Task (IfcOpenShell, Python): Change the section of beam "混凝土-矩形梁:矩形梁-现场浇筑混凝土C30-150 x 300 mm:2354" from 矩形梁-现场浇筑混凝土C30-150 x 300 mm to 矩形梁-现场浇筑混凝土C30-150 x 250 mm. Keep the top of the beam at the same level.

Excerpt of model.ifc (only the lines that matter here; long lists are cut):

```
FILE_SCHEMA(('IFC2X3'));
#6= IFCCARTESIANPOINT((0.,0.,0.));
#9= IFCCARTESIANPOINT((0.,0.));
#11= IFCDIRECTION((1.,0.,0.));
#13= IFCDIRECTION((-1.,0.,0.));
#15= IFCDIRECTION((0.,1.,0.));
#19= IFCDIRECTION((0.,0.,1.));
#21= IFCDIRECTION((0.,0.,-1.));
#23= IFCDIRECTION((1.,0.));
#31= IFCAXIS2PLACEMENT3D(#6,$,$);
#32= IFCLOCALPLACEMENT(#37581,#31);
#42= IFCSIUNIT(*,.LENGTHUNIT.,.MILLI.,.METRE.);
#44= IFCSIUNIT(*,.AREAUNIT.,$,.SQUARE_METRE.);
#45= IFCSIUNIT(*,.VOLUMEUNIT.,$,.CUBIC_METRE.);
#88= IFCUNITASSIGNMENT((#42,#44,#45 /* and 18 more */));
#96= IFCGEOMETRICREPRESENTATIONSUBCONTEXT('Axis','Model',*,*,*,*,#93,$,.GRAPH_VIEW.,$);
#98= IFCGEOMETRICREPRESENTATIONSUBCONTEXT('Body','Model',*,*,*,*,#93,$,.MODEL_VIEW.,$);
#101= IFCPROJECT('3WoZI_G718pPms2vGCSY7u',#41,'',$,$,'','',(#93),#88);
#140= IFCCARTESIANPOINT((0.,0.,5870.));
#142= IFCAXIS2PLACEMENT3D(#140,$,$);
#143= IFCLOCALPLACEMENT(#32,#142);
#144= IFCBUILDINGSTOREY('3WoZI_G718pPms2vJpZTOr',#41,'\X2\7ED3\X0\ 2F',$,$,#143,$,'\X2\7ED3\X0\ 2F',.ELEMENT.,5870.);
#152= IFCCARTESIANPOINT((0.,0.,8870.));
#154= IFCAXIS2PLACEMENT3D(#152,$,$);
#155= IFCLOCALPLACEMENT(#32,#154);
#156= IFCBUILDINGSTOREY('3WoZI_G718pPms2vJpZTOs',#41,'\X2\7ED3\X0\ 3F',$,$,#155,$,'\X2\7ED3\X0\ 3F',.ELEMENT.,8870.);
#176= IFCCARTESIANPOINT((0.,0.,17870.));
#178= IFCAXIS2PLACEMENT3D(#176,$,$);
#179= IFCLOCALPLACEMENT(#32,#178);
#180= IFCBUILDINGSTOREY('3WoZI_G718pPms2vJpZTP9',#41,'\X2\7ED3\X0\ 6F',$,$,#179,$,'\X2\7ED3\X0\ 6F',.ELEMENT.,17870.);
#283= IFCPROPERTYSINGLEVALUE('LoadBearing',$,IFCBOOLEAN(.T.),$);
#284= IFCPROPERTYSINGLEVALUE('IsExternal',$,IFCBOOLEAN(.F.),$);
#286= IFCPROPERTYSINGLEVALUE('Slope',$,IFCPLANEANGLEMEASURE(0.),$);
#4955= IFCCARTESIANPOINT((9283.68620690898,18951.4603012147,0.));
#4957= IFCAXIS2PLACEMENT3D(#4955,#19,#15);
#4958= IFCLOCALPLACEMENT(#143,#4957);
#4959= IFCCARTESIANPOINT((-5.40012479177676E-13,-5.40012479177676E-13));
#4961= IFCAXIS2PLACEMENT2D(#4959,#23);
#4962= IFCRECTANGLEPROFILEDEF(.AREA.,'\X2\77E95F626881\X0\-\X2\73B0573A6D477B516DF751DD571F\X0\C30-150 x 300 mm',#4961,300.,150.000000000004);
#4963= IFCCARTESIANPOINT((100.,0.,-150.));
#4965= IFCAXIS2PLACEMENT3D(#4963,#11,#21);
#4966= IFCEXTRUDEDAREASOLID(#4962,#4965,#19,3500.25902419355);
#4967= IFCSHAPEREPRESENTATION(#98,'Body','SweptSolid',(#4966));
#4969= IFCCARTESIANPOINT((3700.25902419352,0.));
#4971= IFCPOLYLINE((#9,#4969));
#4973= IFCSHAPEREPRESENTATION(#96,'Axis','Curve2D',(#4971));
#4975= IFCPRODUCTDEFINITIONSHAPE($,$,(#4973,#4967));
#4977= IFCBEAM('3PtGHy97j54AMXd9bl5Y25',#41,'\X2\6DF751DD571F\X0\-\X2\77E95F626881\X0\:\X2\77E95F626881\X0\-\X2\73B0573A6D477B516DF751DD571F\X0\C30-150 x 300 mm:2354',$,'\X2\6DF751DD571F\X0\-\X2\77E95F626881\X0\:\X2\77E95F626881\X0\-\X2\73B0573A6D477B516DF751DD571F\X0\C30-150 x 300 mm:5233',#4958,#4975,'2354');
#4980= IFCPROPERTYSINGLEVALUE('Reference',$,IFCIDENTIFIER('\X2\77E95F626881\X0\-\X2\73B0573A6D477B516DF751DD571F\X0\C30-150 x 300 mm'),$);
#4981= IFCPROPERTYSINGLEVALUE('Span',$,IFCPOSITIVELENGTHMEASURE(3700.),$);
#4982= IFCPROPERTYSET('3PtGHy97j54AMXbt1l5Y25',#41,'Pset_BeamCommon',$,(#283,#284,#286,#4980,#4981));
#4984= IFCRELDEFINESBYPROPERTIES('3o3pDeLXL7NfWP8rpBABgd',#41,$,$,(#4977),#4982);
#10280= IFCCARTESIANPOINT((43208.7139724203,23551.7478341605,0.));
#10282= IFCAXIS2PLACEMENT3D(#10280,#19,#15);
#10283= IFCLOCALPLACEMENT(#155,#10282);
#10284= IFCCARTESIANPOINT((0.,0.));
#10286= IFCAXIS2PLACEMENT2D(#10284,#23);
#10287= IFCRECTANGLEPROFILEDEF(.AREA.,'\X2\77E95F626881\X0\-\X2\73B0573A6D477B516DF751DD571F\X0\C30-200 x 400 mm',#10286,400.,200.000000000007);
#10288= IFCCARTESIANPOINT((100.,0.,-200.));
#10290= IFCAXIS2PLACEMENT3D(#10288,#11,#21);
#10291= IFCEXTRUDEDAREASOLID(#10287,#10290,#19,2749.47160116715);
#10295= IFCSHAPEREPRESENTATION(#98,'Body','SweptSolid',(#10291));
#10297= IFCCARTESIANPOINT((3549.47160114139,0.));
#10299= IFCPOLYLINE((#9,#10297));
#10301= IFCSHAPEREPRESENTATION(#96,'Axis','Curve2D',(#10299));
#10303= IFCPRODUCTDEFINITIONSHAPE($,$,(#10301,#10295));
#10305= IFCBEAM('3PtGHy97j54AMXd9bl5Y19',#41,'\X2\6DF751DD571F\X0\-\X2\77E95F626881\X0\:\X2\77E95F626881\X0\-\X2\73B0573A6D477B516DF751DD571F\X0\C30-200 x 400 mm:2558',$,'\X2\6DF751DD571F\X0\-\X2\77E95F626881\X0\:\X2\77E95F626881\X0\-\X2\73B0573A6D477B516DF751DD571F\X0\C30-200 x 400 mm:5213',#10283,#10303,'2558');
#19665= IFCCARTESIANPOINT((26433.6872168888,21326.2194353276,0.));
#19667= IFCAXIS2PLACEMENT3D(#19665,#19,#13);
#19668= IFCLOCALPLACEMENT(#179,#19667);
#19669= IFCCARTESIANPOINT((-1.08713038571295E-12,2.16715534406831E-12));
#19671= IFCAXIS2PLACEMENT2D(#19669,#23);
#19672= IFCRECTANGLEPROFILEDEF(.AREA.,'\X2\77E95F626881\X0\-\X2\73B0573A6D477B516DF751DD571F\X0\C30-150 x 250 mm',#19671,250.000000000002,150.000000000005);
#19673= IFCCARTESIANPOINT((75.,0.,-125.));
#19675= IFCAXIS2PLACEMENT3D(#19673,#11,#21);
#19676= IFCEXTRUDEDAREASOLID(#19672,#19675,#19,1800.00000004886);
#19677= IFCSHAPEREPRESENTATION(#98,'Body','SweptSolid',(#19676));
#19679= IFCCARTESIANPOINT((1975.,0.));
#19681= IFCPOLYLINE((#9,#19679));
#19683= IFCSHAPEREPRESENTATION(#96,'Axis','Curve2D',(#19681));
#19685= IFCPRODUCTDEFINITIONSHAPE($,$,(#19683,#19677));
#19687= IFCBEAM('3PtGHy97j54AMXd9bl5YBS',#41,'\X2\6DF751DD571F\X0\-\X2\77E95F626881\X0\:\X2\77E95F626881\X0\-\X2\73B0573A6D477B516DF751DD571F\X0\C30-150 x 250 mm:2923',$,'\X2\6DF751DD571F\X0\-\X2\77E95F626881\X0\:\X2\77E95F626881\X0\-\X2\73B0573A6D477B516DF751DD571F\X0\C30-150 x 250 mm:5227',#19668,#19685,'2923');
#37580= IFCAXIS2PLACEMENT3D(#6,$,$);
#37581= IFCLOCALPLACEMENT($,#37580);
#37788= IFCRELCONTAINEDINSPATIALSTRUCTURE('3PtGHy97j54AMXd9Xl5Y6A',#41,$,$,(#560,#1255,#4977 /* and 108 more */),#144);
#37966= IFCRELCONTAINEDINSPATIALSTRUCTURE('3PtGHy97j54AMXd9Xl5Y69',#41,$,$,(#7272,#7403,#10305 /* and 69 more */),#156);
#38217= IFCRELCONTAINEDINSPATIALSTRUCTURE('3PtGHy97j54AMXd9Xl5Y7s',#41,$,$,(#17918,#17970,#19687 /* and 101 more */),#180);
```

```python
import ifcopenshell
import ifcopenshell.api.pset
import ifcopenshell.util.element
import ifcopenshell.util.representation

model = ifcopenshell.open("model.ifc")

member = model.by_guid("3PtGHy97j54AMXd9bl5Y25")
source = next(p for p in model.by_type("IfcRectangleProfileDef") if p.ProfileName == "矩形梁-现场浇筑混凝土C30-150 x 250 mm")

body = ifcopenshell.util.representation.get_representation(member, "Model", "Body")
solid = body.Items[0]
old_profile = solid.SweptArea

# Copy the section's sizes but keep this member's own profile position.
profile = ifcopenshell.util.element.copy(model, source)
# Profiles are centred, so shift by half the change in depth to hold the top.
shift = (old_profile.XDim - profile.XDim) / 2
x, y = old_profile.Position.Location.Coordinates
up = (-1.0, 0.0)  # upwards, in the solid's own plane
location = model.createIfcCartesianPoint((x + up[0] * shift, y + up[1] * shift))
profile.Position = model.createIfcAxis2Placement2D(location, old_profile.Position.RefDirection)
solid.SweptArea = profile
if not model.get_total_inverses(old_profile):
    ifcopenshell.util.element.remove_deep2(model, old_profile)
member.Name = member.Name.replace("矩形梁-现场浇筑混凝土C30-150 x 300 mm", "矩形梁-现场浇筑混凝土C30-150 x 250 mm")
member.ObjectType = member.ObjectType.replace("矩形梁-现场浇筑混凝土C30-150 x 300 mm", "矩形梁-现场浇筑混凝土C30-150 x 250 mm")
pset = model.by_id(ifcopenshell.util.element.get_pset(member, "Pset_BeamCommon", should_inherit=False)["id"])
ifcopenshell.api.pset.edit_pset(model, pset=pset, properties={"Reference": "矩形梁-现场浇筑混凝土C30-150 x 250 mm"})

print(solid.SweptArea)

model.write("model_updated.ifc")
```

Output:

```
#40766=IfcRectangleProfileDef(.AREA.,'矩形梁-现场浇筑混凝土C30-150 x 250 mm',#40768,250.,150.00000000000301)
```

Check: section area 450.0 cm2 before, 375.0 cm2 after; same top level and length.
